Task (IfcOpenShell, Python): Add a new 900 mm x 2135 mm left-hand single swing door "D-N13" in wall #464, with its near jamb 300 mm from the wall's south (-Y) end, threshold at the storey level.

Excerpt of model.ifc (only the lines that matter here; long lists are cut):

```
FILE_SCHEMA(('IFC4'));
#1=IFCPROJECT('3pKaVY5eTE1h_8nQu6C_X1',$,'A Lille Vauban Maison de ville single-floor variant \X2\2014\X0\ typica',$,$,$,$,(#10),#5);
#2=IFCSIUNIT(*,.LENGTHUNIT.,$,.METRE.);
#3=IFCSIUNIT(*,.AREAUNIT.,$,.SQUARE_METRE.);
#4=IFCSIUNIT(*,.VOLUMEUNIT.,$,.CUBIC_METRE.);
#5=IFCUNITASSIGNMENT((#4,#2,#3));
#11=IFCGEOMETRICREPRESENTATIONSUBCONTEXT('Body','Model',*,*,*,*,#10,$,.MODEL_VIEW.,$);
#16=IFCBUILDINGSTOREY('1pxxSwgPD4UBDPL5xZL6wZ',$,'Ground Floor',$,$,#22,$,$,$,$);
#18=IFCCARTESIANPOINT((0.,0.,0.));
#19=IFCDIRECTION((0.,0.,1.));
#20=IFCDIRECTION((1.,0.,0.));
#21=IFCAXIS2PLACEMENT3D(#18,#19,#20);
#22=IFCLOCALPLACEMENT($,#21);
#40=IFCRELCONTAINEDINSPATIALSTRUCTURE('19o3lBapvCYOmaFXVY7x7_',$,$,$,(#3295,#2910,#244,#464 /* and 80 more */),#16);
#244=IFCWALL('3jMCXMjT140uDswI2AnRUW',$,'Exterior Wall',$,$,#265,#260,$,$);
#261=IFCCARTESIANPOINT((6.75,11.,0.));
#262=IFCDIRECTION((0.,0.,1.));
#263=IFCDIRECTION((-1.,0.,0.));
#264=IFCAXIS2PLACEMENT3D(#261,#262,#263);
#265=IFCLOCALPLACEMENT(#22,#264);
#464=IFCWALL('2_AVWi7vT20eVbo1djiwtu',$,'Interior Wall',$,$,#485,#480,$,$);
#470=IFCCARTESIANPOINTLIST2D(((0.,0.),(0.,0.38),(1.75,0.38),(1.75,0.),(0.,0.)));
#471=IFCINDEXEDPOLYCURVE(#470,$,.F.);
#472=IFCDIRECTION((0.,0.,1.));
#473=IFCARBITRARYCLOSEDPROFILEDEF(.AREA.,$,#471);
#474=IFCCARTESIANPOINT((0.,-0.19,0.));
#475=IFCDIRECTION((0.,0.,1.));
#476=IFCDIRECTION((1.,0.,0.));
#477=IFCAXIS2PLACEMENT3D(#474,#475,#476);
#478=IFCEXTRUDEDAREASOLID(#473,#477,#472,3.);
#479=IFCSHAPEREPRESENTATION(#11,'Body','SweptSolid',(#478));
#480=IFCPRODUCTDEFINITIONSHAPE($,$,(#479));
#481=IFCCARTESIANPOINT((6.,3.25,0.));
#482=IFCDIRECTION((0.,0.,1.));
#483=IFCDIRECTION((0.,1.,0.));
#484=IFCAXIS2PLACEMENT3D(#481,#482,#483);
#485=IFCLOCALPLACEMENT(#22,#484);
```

```python
import numpy as np
import ifcopenshell
import ifcopenshell.api.feature
import ifcopenshell.api.geometry
import ifcopenshell.api.root
import ifcopenshell.api.spatial
import ifcopenshell.geom
import ifcopenshell.util.element
import ifcopenshell.util.placement
import ifcopenshell.util.representation
import ifcopenshell.util.shape
import ifcopenshell.util.unit

model = ifcopenshell.open("model.ifc")
unit_scale = ifcopenshell.util.unit.calculate_unit_scale(model)
settings = ifcopenshell.geom.settings()


def volume(element):
    """Net volume in cubic metres, openings subtracted."""
    shape = ifcopenshell.geom.create_shape(settings, element)
    return ifcopenshell.util.shape.get_volume(shape.geometry)


wall = model.by_guid("2_AVWi7vT20eVbo1djiwtu")
storey = ifcopenshell.util.element.get_container(wall, ifc_class="IfcBuildingStorey")
context = ifcopenshell.util.representation.get_context(model, "Model", "Body", "MODEL_VIEW")
before = volume(wall)

width, height, from_end, sill = 0.9, 2.135, 0.3, 0.0  # metres

# The wall runs along its own X axis, and the end named is its -X end.
wall_shape = ifcopenshell.geom.create_shape(settings, wall)
x, y, z = ifcopenshell.util.shape.get_vertices(wall_shape.geometry).T
start = x.min() + from_end
face, thickness = float(y.min()), float(y.max() - y.min())
wall_matrix = ifcopenshell.util.placement.get_local_placement(wall.ObjectPlacement)
level = ifcopenshell.util.placement.get_local_placement(storey.ObjectPlacement)[2, 3]


def in_wall(x, y):
    """Placement at x, y metres in the wall's axes, at sill height."""
    matrix = wall_matrix.copy()
    matrix[:, 3] = wall_matrix @ np.array([x / unit_scale, y / unit_scale, 0.0, 1.0])
    matrix[2, 3] = level + sill / unit_scale
    return matrix


# Opening: a box that overshoots both wall faces by 50 mm.
opening = ifcopenshell.api.root.create_entity(model, ifc_class="IfcOpeningElement", predefined_type="OPENING")
box = ifcopenshell.api.geometry.add_wall_representation(
    model, context=context, length=width, height=height, thickness=thickness + 0.1
)
ifcopenshell.api.geometry.assign_representation(model, product=opening, representation=box)
ifcopenshell.api.geometry.edit_object_placement(model, product=opening, matrix=in_wall(start, face - 0.05), is_si=False)
ifcopenshell.api.feature.add_feature(model, feature=opening, element=wall)

door = ifcopenshell.api.root.create_entity(model, ifc_class="IfcDoor", name="D-N13", predefined_type="DOOR")
door.OverallWidth, door.OverallHeight = width / unit_scale, height / unit_scale
door.OperationType = "SINGLE_SWING_LEFT"
body = ifcopenshell.api.geometry.add_door_representation(
    model,
    context=context,
    overall_width=door.OverallWidth,
    overall_height=door.OverallHeight,
    operation_type="SINGLE_SWING_LEFT",
    lining_properties={"LiningDepth": thickness / unit_scale, "ThresholdDepth": thickness / unit_scale},
)
ifcopenshell.api.geometry.assign_representation(model, product=door, representation=body)
ifcopenshell.api.spatial.assign_container(model, products=[door], relating_structure=storey)
ifcopenshell.api.feature.add_filling(model, opening=opening, element=door)

# The lining spans the wall, so the door starts at the wall face.
ifcopenshell.api.geometry.edit_object_placement(model, product=door, matrix=in_wall(start, face), is_si=False)

after = volume(wall)

print(f"wall volume {before:.3f} -> {after:.3f} m3")

model.write("model_v2.ifc")
```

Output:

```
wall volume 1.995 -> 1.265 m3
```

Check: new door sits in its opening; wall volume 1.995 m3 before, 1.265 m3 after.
